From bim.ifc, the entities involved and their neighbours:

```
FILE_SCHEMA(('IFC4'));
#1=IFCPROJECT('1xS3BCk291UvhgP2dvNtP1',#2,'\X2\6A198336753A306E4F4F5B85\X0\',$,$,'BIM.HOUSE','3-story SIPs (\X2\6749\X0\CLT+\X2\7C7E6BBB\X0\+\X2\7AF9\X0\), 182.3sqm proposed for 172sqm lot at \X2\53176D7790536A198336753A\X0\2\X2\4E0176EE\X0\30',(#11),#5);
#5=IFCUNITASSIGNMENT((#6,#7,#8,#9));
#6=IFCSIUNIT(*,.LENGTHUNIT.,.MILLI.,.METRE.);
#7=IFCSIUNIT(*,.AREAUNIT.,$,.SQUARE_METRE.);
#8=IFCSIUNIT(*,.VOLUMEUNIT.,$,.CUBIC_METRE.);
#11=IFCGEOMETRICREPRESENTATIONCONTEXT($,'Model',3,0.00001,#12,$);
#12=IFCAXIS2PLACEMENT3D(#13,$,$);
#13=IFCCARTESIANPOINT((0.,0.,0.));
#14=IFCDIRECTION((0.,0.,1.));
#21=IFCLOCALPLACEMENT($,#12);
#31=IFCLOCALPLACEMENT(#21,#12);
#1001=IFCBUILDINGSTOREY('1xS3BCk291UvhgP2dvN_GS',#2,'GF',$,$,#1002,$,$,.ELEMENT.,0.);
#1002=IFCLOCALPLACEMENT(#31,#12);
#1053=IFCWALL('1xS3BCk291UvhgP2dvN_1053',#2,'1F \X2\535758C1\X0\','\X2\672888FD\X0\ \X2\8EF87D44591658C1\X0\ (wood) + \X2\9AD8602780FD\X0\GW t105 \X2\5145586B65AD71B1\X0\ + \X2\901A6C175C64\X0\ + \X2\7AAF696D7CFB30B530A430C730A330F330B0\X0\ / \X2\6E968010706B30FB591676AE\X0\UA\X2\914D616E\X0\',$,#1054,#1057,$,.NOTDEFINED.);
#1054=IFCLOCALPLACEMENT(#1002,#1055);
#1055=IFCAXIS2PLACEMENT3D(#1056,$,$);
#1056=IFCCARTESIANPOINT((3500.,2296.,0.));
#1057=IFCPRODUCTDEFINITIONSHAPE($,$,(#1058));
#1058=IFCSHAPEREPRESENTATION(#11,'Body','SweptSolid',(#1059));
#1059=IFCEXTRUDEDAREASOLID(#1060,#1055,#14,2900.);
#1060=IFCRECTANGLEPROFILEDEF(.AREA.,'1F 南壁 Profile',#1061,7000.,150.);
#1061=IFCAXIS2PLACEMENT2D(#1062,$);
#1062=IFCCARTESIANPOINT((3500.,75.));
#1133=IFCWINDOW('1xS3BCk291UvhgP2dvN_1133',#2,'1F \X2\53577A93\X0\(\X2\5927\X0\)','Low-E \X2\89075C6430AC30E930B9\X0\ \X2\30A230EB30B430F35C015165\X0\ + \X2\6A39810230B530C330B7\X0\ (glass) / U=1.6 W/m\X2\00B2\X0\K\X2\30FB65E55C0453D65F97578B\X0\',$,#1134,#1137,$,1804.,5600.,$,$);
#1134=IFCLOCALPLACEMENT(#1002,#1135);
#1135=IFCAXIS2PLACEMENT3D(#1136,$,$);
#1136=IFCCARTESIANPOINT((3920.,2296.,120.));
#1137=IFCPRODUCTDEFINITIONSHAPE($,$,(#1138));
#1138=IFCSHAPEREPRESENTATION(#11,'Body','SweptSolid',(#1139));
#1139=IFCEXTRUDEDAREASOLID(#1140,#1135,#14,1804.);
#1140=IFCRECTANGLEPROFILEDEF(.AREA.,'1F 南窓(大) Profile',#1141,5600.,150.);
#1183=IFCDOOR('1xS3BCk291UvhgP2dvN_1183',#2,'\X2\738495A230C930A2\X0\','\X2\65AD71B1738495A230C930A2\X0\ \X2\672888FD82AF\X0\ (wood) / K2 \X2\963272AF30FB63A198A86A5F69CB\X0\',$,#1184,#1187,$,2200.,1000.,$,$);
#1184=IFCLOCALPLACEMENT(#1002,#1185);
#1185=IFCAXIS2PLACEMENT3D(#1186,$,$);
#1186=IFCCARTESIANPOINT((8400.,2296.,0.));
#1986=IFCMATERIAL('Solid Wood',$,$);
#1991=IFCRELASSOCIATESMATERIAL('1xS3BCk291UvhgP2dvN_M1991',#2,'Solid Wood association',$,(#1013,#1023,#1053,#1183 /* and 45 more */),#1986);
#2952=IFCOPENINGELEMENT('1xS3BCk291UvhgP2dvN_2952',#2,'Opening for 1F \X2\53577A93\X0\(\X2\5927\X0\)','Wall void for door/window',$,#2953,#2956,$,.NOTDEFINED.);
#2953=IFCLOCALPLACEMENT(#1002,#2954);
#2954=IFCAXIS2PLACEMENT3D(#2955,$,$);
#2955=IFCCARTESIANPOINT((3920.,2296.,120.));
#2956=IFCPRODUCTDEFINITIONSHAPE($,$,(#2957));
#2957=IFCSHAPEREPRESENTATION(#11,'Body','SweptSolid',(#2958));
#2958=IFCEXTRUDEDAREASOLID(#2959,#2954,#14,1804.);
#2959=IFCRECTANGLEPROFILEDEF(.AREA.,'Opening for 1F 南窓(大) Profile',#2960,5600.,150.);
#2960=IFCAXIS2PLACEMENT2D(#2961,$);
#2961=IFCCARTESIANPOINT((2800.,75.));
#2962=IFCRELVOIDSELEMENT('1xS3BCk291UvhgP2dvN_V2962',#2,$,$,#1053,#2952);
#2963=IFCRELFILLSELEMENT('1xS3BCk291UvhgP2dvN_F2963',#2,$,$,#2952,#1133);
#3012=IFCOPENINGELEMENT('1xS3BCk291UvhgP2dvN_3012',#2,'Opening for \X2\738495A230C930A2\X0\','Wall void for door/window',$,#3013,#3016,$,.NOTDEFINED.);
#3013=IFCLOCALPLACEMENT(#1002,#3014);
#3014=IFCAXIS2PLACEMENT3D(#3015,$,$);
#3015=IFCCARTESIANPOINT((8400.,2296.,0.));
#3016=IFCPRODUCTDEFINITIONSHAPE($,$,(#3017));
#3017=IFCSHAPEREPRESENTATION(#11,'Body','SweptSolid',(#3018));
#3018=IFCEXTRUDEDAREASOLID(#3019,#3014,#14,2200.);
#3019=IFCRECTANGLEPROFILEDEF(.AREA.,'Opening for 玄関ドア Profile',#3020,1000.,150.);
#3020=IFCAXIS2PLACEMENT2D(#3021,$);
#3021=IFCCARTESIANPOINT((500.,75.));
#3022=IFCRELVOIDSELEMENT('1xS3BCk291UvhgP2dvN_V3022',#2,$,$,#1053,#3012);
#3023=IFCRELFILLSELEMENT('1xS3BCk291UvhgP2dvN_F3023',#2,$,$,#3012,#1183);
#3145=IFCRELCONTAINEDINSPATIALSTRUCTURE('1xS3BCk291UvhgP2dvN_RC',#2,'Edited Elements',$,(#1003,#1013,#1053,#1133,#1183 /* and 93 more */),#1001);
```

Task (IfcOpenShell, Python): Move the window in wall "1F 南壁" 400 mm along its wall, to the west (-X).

```python
import ifcopenshell
import ifcopenshell.api.geometry
import ifcopenshell.util.placement

model = ifcopenshell.open("bim.ifc")

window = model.by_guid("1xS3BCk291UvhgP2dvN_1133")
opening = window.FillsVoids[0].RelatingOpeningElement
wall = opening.VoidsElements[0].RelatingBuildingElement

wall_matrix = ifcopenshell.util.placement.get_local_placement(wall.ObjectPlacement)
shift = wall_matrix[:3, 0] * -400.0
before = ifcopenshell.util.placement.get_local_placement(window.ObjectPlacement)[:3, 3].copy()

# The window is not placed relative to its opening, so move both.
for product in (opening, window):
    matrix = ifcopenshell.util.placement.get_local_placement(product.ObjectPlacement)
    matrix[:3, 3] += shift
    ifcopenshell.api.geometry.edit_object_placement(model, product=product, matrix=matrix, is_si=False)

after = ifcopenshell.util.placement.get_local_placement(window.ObjectPlacement)[:3, 3]
print("window moved by", (after - before).round(3) + 0.0)

model.write("bim_rev.ifc")
```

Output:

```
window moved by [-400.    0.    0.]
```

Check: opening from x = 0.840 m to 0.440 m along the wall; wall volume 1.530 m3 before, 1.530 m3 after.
